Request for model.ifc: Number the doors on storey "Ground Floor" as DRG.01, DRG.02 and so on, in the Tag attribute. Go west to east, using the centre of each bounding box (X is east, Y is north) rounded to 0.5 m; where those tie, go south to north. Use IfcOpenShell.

First a look at what the model holds.

```python
import ifcopenshell
import ifcopenshell.util.element
import ifcopenshell.util.placement

model = ifcopenshell.open("model.ifc")
print(model.schema)
storey = next(s for s in model.by_type("IfcBuildingStorey") if s.Name == "Ground Floor")
doors = [e for e in ifcopenshell.util.element.get_decomposition(storey) if e.is_a("IfcDoor")]
for e in sorted(doors, key=lambda e: e.id()):
    origin = ifcopenshell.util.placement.get_local_placement(e.ObjectPlacement)[:3, 3]
    print(e.id(), e.Tag, e.Name, origin.round(2) + 0.0, sep=" | ")
```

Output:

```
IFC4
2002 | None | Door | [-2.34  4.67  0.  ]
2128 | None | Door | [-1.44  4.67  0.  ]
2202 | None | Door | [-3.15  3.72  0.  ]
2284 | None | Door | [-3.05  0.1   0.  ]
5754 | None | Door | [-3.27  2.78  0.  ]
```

```python
import ifcopenshell
import ifcopenshell.geom
import ifcopenshell.util.element
import ifcopenshell.util.shape

model = ifcopenshell.open("model.ifc")
settings = ifcopenshell.geom.settings()
settings.set("use-world-coords", True)


def centre(element):
    shape = ifcopenshell.geom.create_shape(settings, element)
    return ifcopenshell.util.shape.get_bbox_centroid(shape.geometry)


storey = next(s for s in model.by_type("IfcBuildingStorey") if s.Name == "Ground Floor")
doors = [e for e in ifcopenshell.util.element.get_decomposition(storey) if e.is_a("IfcDoor")]

# Insertion points can sit at a corner or the storey origin, so sort by the geometry (in metres).
centres = {e: centre(e) for e in doors}
doors.sort(key=lambda e: (round(centres[e][0] / 0.5), centres[e][1]))

for i, e in enumerate(doors, start=1):
    number = f"DRG.{i:02d}"
    e.Tag = number
    print(e.id(), number)

model.write("model_rev.ifc")
```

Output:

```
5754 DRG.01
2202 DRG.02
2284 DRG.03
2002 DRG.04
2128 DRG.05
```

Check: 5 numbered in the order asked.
